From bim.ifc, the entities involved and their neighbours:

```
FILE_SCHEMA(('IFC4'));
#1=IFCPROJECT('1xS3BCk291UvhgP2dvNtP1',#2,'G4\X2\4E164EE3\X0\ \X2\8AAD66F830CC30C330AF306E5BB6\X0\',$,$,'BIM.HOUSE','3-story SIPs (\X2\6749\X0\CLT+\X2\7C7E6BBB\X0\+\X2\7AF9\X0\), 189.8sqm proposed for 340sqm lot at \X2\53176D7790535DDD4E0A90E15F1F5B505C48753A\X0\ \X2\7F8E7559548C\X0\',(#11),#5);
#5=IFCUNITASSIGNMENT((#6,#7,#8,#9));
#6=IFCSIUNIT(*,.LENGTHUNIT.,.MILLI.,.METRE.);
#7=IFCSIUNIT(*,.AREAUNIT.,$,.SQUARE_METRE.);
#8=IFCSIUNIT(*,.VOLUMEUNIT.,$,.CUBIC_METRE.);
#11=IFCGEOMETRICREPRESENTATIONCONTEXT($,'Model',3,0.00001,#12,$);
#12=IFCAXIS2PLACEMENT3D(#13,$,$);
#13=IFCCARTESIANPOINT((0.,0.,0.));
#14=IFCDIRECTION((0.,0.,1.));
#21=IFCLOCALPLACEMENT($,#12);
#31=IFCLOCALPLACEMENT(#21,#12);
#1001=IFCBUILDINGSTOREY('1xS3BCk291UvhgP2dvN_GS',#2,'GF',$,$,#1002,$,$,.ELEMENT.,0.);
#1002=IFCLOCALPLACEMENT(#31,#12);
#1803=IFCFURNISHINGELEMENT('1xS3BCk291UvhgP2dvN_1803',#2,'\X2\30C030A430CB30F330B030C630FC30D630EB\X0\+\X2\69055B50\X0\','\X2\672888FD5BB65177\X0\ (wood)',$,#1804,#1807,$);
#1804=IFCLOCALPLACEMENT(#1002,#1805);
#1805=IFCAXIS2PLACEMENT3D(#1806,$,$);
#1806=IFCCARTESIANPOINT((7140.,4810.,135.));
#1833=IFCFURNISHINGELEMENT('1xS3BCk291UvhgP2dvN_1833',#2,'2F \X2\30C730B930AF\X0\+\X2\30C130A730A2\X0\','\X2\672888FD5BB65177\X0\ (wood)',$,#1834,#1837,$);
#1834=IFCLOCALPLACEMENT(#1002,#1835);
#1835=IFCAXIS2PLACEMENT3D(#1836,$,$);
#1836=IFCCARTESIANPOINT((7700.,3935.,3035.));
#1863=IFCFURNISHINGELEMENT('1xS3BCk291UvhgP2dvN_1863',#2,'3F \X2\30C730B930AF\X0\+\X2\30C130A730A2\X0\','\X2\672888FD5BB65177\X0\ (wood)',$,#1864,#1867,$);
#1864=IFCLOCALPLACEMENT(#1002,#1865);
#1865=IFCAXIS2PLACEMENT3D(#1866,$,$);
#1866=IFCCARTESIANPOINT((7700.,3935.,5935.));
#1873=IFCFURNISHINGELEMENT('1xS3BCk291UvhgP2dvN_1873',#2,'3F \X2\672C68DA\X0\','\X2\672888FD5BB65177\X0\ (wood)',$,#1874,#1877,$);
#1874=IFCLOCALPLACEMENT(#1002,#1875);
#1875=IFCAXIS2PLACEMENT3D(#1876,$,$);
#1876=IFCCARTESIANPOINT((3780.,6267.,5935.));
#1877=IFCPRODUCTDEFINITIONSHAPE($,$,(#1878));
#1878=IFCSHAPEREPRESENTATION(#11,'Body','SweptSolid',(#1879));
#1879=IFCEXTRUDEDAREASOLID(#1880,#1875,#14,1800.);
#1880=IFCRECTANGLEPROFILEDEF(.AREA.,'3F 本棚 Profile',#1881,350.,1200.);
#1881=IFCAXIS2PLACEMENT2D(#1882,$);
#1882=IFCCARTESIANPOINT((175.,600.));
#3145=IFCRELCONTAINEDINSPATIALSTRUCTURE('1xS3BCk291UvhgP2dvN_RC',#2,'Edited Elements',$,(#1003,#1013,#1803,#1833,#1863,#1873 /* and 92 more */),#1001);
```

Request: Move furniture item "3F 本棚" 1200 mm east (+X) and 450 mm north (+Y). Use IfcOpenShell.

```python
import ifcopenshell
import ifcopenshell.api.geometry
import ifcopenshell.util.placement

model = ifcopenshell.open("bim.ifc")

item = model.by_guid("1xS3BCk291UvhgP2dvN_1873")
matrix = ifcopenshell.util.placement.get_local_placement(item.ObjectPlacement)
matrix[0, 3] += 1200.0
matrix[1, 3] += 450.0
ifcopenshell.api.geometry.edit_object_placement(model, product=item, matrix=matrix, is_si=False)

print(ifcopenshell.util.placement.get_local_placement(item.ObjectPlacement).round(3) + 0.0)

model.write("bim_v2.ifc")
```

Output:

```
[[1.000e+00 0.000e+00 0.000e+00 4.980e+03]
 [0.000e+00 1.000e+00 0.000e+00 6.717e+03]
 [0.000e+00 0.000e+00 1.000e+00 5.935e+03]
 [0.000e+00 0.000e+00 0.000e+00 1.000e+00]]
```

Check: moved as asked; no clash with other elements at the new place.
